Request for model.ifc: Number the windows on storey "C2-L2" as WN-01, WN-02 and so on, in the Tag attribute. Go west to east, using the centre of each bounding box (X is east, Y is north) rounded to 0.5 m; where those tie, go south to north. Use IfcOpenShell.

First a look at what the model holds.

```python
import ifcopenshell
import ifcopenshell.util.element
import ifcopenshell.util.placement

model = ifcopenshell.open("model.ifc")
print(model.schema)
storey = next(s for s in model.by_type("IfcBuildingStorey") if s.Name == "C2-L2")
windows = [e for e in ifcopenshell.util.element.get_decomposition(storey) if e.is_a("IfcWindow")]
for e in sorted(windows, key=lambda e: e.id()):
    origin = ifcopenshell.util.placement.get_local_placement(e.ObjectPlacement)[:3, 3]
    print(e.id(), e.Tag, e.Name, origin.round(2) + 0.0, sep=" | ")
```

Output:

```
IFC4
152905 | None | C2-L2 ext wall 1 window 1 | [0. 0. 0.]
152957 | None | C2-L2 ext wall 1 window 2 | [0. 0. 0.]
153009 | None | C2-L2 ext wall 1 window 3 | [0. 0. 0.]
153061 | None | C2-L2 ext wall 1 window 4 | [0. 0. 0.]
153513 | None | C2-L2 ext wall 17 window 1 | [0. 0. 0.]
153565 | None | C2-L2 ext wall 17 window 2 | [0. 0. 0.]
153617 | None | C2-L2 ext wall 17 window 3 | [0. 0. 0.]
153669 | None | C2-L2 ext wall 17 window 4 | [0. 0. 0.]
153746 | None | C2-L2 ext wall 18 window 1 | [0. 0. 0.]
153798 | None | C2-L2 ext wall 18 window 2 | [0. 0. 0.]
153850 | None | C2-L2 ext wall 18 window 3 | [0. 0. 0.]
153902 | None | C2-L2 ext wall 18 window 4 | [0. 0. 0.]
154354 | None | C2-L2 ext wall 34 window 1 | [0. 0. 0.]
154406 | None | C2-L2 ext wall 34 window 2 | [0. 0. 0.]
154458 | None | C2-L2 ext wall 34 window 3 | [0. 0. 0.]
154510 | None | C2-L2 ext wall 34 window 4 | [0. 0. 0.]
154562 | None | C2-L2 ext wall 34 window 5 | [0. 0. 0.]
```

```python
import ifcopenshell
import ifcopenshell.geom
import ifcopenshell.util.element
import ifcopenshell.util.shape

model = ifcopenshell.open("model.ifc")
settings = ifcopenshell.geom.settings()
settings.set("use-world-coords", True)


def centre(element):
    shape = ifcopenshell.geom.create_shape(settings, element)
    return ifcopenshell.util.shape.get_bbox_centroid(shape.geometry)


storey = next(s for s in model.by_type("IfcBuildingStorey") if s.Name == "C2-L2")
windows = [e for e in ifcopenshell.util.element.get_decomposition(storey) if e.is_a("IfcWindow")]

# Insertion points can sit at a corner or the storey origin, so sort by the geometry (in metres).
centres = {e: centre(e) for e in windows}
windows.sort(key=lambda e: (round(centres[e][0] / 0.5), centres[e][1]))

for i, e in enumerate(windows, start=1):
    number = f"WN-{i:02d}"
    e.Tag = number
    print(e.id(), number)

model.write("model_rev.ifc")
```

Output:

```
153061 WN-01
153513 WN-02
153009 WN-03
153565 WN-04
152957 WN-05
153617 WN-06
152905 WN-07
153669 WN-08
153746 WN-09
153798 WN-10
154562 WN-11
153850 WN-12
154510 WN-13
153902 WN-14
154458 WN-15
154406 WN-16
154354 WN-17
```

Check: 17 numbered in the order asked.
